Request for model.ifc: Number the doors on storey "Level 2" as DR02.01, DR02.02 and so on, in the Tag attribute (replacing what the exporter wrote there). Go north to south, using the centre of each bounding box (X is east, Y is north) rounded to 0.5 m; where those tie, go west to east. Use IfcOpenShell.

First a look at what the model holds.

```python
import ifcopenshell
import ifcopenshell.util.element
import ifcopenshell.util.placement

model = ifcopenshell.open("model.ifc")
print(model.schema)
storey = next(s for s in model.by_type("IfcBuildingStorey") if s.Name == "Level 2")
doors = [e for e in ifcopenshell.util.element.get_decomposition(storey) if e.is_a("IfcDoor")]
for e in sorted(doors, key=lambda e: e.id()):
    origin = ifcopenshell.util.placement.get_local_placement(e.ObjectPlacement)[:3, 3]
    print(e.id(), e.Tag, e.Name, origin.round(2) + 0.0, sep=" | ")
```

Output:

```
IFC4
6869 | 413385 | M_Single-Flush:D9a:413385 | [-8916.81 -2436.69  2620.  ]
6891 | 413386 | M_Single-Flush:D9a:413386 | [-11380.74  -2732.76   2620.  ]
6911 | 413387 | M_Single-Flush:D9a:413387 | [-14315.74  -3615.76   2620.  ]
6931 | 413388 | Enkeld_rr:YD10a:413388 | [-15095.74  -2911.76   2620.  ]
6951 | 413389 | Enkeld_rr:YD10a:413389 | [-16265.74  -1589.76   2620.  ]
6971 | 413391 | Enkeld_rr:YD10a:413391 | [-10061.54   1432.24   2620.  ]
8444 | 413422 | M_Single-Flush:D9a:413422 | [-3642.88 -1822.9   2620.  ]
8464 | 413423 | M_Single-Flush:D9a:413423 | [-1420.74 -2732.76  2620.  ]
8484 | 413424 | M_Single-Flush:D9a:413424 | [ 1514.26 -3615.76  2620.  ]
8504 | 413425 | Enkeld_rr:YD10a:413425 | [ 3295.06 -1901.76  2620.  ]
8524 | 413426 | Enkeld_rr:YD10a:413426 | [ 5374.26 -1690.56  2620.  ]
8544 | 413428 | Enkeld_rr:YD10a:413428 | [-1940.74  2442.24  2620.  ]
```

```python
import ifcopenshell
import ifcopenshell.geom
import ifcopenshell.util.element
import ifcopenshell.util.shape

model = ifcopenshell.open("model.ifc")
settings = ifcopenshell.geom.settings()
settings.set("use-world-coords", True)


def centre(element):
    shape = ifcopenshell.geom.create_shape(settings, element)
    return ifcopenshell.util.shape.get_bbox_centroid(shape.geometry)


storey = next(s for s in model.by_type("IfcBuildingStorey") if s.Name == "Level 2")
doors = [e for e in ifcopenshell.util.element.get_decomposition(storey) if e.is_a("IfcDoor")]

# Insertion points can sit at a corner or the storey origin, so sort by the geometry (in metres).
centres = {e: centre(e) for e in doors}
doors.sort(key=lambda e: (-round(centres[e][1] / 0.5), centres[e][0]))

for i, e in enumerate(doors, start=1):
    number = f"DR02.{i:02d}"
    e.Tag = number
    print(e.id(), number)

model.write("model_edited.ifc")
```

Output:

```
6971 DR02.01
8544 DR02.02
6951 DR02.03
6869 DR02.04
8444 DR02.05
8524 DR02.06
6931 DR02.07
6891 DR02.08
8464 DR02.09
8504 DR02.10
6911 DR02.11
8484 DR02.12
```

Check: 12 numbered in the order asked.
